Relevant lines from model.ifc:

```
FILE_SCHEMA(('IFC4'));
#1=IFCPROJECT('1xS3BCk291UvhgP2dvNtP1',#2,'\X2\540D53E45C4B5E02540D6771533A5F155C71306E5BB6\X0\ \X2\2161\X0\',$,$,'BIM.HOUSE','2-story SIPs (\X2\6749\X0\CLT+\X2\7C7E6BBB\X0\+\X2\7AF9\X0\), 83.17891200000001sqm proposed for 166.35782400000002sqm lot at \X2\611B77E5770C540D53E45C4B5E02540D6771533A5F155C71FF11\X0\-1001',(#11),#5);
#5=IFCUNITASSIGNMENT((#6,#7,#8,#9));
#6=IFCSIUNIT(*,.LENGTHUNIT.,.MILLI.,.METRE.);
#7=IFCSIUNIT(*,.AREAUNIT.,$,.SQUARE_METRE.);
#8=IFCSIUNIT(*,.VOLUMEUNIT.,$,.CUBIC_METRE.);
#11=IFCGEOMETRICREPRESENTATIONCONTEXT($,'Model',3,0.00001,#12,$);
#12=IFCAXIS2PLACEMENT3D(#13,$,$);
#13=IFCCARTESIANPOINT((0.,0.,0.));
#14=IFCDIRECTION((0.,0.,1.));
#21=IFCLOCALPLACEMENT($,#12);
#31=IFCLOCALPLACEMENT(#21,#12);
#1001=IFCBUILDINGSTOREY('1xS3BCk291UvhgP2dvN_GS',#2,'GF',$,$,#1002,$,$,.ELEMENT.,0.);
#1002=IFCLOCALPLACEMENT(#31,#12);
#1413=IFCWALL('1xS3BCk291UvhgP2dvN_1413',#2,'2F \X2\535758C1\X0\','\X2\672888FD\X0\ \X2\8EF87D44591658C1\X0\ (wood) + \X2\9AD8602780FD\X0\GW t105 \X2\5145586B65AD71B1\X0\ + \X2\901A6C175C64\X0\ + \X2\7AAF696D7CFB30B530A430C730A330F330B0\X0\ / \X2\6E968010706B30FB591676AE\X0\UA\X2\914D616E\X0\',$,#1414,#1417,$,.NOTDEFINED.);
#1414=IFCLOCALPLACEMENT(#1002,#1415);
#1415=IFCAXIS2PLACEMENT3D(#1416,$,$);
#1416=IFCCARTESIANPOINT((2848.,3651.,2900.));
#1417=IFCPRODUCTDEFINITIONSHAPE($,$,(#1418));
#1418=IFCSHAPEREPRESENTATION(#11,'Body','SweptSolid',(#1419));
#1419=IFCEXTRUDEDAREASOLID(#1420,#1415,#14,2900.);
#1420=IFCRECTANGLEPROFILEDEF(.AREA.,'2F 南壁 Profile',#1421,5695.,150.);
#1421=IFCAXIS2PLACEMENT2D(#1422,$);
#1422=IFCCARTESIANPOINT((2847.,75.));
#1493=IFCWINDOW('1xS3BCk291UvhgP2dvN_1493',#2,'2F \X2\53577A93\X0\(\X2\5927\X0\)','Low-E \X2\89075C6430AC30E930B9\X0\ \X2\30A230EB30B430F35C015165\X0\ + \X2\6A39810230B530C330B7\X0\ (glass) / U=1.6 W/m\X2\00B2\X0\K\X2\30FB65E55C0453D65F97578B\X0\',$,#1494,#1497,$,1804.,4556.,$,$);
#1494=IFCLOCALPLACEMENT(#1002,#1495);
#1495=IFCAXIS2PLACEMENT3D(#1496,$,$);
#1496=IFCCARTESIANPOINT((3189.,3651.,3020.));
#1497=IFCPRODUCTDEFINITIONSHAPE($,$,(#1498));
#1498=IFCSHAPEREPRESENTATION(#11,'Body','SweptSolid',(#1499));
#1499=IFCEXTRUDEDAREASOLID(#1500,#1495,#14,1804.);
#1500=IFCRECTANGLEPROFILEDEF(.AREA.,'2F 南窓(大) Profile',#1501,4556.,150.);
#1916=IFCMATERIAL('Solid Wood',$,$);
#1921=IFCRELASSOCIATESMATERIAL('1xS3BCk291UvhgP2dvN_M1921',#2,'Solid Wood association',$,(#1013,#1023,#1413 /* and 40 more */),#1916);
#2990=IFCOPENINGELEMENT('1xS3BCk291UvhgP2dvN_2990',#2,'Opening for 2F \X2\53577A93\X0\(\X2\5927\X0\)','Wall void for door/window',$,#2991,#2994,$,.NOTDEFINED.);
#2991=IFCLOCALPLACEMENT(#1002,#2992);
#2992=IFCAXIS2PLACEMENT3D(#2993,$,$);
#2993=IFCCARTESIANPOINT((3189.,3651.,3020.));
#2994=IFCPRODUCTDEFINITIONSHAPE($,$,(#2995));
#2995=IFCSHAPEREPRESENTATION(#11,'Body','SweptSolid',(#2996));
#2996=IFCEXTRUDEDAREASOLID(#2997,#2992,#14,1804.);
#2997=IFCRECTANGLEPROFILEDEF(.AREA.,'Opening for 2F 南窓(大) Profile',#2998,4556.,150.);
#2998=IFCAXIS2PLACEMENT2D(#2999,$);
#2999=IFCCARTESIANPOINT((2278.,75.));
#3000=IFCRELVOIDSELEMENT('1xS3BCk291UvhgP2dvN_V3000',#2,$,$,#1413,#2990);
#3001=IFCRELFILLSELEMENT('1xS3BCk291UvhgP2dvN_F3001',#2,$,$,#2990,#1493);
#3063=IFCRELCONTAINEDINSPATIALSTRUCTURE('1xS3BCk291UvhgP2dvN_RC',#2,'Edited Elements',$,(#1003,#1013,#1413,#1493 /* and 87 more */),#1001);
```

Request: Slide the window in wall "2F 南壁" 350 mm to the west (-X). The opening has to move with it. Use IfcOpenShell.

```python
import ifcopenshell
import ifcopenshell.api.geometry
import ifcopenshell.util.placement

model = ifcopenshell.open("model.ifc")

window = model.by_guid("1xS3BCk291UvhgP2dvN_1493")
opening = window.FillsVoids[0].RelatingOpeningElement
wall = opening.VoidsElements[0].RelatingBuildingElement

wall_matrix = ifcopenshell.util.placement.get_local_placement(wall.ObjectPlacement)
shift = wall_matrix[:3, 0] * -350.0
before = ifcopenshell.util.placement.get_local_placement(window.ObjectPlacement)[:3, 3].copy()

# The window is not placed relative to its opening, so move both.
for product in (opening, window):
    matrix = ifcopenshell.util.placement.get_local_placement(product.ObjectPlacement)
    matrix[:3, 3] += shift
    ifcopenshell.api.geometry.edit_object_placement(model, product=product, matrix=matrix, is_si=False)

after = ifcopenshell.util.placement.get_local_placement(window.ObjectPlacement)[:3, 3]
print("window moved by", (after - before).round(3) + 0.0)

model.write("model-out.ifc")
```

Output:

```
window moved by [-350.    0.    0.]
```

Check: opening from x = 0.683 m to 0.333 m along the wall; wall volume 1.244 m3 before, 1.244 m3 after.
